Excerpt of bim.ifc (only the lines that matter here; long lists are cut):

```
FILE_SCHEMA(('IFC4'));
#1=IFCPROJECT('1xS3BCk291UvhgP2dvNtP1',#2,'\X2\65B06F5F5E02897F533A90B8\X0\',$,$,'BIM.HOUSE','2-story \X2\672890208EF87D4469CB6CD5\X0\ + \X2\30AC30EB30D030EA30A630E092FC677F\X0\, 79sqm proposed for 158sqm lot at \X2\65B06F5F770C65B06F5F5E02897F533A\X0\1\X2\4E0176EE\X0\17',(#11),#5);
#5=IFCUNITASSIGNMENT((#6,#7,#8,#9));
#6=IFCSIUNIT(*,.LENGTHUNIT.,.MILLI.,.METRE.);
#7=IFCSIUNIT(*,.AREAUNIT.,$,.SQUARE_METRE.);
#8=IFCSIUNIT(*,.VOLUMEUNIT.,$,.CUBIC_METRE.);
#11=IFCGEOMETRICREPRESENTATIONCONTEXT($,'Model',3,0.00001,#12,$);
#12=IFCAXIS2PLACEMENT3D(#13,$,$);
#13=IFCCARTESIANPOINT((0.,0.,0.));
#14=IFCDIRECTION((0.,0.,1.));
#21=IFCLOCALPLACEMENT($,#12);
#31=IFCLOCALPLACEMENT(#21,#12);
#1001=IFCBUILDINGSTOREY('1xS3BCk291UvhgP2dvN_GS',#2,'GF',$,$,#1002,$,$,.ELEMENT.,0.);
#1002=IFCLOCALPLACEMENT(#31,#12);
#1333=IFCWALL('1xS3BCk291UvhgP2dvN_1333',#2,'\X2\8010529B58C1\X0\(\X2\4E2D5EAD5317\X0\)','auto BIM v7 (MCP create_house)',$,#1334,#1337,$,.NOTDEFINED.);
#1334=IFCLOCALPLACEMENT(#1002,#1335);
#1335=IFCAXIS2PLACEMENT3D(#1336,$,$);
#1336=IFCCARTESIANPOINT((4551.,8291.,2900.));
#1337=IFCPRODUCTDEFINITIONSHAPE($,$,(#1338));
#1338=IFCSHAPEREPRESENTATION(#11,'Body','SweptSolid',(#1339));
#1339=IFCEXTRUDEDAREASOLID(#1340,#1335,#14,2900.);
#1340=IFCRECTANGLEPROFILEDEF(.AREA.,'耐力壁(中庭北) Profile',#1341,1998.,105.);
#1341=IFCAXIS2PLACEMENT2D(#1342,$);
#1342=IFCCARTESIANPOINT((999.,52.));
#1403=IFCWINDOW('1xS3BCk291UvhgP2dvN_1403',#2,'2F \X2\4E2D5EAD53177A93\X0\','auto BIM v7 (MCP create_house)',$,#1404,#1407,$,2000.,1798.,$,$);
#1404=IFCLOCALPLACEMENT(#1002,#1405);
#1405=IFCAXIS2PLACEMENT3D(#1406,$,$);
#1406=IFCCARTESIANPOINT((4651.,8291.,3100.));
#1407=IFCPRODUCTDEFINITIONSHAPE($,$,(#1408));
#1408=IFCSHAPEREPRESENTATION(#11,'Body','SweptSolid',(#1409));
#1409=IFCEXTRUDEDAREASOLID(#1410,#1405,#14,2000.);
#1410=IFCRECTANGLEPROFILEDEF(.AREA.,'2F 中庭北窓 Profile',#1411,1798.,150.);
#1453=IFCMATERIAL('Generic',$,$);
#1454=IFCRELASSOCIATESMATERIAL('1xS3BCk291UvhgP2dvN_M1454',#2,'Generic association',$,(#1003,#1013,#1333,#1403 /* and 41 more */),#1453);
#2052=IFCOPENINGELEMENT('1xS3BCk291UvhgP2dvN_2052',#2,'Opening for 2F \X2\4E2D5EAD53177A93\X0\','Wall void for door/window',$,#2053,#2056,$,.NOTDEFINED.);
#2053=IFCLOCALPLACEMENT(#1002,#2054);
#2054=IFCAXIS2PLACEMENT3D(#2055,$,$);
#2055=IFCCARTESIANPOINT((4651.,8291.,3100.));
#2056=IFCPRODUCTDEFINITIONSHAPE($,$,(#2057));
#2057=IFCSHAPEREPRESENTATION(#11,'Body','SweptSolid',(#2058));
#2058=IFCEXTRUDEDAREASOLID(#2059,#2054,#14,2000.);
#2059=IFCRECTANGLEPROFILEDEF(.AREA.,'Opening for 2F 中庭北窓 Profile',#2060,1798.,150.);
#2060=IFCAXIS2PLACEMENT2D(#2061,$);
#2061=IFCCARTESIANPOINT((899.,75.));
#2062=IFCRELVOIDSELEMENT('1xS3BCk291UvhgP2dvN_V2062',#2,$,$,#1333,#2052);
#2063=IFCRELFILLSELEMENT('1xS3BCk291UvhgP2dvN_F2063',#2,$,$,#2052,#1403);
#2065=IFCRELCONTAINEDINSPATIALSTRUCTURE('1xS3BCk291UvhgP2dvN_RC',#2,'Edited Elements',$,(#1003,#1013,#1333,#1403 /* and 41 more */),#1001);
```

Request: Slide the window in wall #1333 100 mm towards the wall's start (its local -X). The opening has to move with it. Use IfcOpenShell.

```python
import ifcopenshell
import ifcopenshell.api.geometry
import ifcopenshell.util.placement
import ifcopenshell.util.unit

model = ifcopenshell.open("bim.ifc")
unit_scale = ifcopenshell.util.unit.calculate_unit_scale(model)

window = model.by_id(1403)
opening = window.FillsVoids[0].RelatingOpeningElement
wall = opening.VoidsElements[0].RelatingBuildingElement

wall_matrix = ifcopenshell.util.placement.get_local_placement(wall.ObjectPlacement)
shift = wall_matrix[:3, 0] * -0.1 / unit_scale
before = ifcopenshell.util.placement.get_local_placement(window.ObjectPlacement)[:3, 3].copy()

# The window is not placed relative to its opening, so move both.
for product in (opening, window):
    matrix = ifcopenshell.util.placement.get_local_placement(product.ObjectPlacement)
    matrix[:3, 3] += shift
    ifcopenshell.api.geometry.edit_object_placement(model, product=product, matrix=matrix, is_si=False)

after = ifcopenshell.util.placement.get_local_placement(window.ObjectPlacement)[:3, 3]
print("window moved by", (after - before).round(3) + 0.0)

model.write("bim_v2.ifc")
```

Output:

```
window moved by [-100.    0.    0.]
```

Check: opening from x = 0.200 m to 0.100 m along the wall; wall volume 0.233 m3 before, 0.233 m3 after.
